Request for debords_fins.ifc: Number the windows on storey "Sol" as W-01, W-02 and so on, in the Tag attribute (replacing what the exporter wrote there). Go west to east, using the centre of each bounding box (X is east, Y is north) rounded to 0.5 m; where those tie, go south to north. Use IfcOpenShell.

First a look at what the model holds.

```python
import ifcopenshell
import ifcopenshell.util.element
import ifcopenshell.util.placement

model = ifcopenshell.open("debords_fins.ifc")
print(model.schema)
storey = next(s for s in model.by_type("IfcBuildingStorey") if s.Name == "Sol")
windows = [e for e in ifcopenshell.util.element.get_decomposition(storey) if e.is_a("IfcWindow")]
for e in sorted(windows, key=lambda e: e.id()):
    origin = ifcopenshell.util.placement.get_local_placement(e.ObjectPlacement)[:3, 3]
    print(e.id(), e.Tag, e.Name, origin.round(2) + 0.0, sep=" | ")
```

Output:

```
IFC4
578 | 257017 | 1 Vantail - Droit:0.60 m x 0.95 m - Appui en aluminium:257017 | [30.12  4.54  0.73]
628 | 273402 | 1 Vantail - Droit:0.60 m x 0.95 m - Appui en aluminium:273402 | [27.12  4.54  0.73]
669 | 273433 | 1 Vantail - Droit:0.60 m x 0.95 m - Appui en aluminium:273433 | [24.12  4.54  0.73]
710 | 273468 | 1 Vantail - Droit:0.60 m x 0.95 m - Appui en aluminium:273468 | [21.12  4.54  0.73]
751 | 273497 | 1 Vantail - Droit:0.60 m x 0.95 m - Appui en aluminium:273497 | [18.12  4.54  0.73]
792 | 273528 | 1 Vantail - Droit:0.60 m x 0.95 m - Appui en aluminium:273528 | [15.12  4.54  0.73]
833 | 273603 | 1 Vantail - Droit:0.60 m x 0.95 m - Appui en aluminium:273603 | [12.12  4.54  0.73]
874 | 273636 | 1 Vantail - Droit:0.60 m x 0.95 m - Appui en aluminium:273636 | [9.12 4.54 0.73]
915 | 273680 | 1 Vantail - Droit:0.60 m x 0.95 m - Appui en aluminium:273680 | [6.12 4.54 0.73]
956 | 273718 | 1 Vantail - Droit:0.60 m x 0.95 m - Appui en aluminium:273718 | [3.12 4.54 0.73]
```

```python
import ifcopenshell
import ifcopenshell.geom
import ifcopenshell.util.element
import ifcopenshell.util.shape

model = ifcopenshell.open("debords_fins.ifc")
settings = ifcopenshell.geom.settings()
settings.set("use-world-coords", True)


def centre(element):
    shape = ifcopenshell.geom.create_shape(settings, element)
    return ifcopenshell.util.shape.get_bbox_centroid(shape.geometry)


storey = next(s for s in model.by_type("IfcBuildingStorey") if s.Name == "Sol")
windows = [e for e in ifcopenshell.util.element.get_decomposition(storey) if e.is_a("IfcWindow")]

# Insertion points can sit at a corner or the storey origin, so sort by the geometry (in metres).
centres = {e: centre(e) for e in windows}
windows.sort(key=lambda e: (round(centres[e][0] / 0.5), centres[e][1]))

for i, e in enumerate(windows, start=1):
    number = f"W-{i:02d}"
    e.Tag = number
    print(e.id(), number)

model.write("debords_fins_updated.ifc")
```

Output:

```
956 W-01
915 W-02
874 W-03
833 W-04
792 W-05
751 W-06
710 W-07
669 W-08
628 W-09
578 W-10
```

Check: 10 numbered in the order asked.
